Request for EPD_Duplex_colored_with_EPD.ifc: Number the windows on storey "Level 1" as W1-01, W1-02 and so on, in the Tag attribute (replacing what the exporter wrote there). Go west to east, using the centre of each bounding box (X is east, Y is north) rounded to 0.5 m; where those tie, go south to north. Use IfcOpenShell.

First a look at what the model holds.

```python
import ifcopenshell
import ifcopenshell.util.element
import ifcopenshell.util.placement

model = ifcopenshell.open("EPD_Duplex_colored_with_EPD.ifc")
print(model.schema)
storey = next(s for s in model.by_type("IfcBuildingStorey") if s.Name == "Level 1")
windows = [e for e in ifcopenshell.util.element.get_decomposition(storey) if e.is_a("IfcWindow")]
for e in sorted(windows, key=lambda e: e.id()):
    origin = ifcopenshell.util.placement.get_local_placement(e.ObjectPlacement)[:3, 3]
    print(e.id(), e.Tag, e.Name, origin.round(2) + 0.0, sep=" | ")
```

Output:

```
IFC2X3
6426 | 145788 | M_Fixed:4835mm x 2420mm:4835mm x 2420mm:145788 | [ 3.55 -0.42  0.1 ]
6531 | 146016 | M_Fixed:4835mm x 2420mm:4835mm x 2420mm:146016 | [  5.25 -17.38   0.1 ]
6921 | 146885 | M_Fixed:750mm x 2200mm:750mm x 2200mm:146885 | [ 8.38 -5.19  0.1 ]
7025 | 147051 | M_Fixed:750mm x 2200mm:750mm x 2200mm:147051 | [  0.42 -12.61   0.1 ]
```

```python
import ifcopenshell
import ifcopenshell.geom
import ifcopenshell.util.element
import ifcopenshell.util.shape

model = ifcopenshell.open("EPD_Duplex_colored_with_EPD.ifc")
settings = ifcopenshell.geom.settings()
settings.set("use-world-coords", True)


def centre(element):
    shape = ifcopenshell.geom.create_shape(settings, element)
    return ifcopenshell.util.shape.get_bbox_centroid(shape.geometry)


storey = next(s for s in model.by_type("IfcBuildingStorey") if s.Name == "Level 1")
windows = [e for e in ifcopenshell.util.element.get_decomposition(storey) if e.is_a("IfcWindow")]

# Insertion points can sit at a corner or the storey origin, so sort by the geometry (in metres).
centres = {e: centre(e) for e in windows}
windows.sort(key=lambda e: (round(centres[e][0] / 0.5), centres[e][1]))

for i, e in enumerate(windows, start=1):
    number = f"W1-{i:02d}"
    e.Tag = number
    print(e.id(), number)

model.write("EPD_Duplex_colored_with_EPD_updated.ifc")
```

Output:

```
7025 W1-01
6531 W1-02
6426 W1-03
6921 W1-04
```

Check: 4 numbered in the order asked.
